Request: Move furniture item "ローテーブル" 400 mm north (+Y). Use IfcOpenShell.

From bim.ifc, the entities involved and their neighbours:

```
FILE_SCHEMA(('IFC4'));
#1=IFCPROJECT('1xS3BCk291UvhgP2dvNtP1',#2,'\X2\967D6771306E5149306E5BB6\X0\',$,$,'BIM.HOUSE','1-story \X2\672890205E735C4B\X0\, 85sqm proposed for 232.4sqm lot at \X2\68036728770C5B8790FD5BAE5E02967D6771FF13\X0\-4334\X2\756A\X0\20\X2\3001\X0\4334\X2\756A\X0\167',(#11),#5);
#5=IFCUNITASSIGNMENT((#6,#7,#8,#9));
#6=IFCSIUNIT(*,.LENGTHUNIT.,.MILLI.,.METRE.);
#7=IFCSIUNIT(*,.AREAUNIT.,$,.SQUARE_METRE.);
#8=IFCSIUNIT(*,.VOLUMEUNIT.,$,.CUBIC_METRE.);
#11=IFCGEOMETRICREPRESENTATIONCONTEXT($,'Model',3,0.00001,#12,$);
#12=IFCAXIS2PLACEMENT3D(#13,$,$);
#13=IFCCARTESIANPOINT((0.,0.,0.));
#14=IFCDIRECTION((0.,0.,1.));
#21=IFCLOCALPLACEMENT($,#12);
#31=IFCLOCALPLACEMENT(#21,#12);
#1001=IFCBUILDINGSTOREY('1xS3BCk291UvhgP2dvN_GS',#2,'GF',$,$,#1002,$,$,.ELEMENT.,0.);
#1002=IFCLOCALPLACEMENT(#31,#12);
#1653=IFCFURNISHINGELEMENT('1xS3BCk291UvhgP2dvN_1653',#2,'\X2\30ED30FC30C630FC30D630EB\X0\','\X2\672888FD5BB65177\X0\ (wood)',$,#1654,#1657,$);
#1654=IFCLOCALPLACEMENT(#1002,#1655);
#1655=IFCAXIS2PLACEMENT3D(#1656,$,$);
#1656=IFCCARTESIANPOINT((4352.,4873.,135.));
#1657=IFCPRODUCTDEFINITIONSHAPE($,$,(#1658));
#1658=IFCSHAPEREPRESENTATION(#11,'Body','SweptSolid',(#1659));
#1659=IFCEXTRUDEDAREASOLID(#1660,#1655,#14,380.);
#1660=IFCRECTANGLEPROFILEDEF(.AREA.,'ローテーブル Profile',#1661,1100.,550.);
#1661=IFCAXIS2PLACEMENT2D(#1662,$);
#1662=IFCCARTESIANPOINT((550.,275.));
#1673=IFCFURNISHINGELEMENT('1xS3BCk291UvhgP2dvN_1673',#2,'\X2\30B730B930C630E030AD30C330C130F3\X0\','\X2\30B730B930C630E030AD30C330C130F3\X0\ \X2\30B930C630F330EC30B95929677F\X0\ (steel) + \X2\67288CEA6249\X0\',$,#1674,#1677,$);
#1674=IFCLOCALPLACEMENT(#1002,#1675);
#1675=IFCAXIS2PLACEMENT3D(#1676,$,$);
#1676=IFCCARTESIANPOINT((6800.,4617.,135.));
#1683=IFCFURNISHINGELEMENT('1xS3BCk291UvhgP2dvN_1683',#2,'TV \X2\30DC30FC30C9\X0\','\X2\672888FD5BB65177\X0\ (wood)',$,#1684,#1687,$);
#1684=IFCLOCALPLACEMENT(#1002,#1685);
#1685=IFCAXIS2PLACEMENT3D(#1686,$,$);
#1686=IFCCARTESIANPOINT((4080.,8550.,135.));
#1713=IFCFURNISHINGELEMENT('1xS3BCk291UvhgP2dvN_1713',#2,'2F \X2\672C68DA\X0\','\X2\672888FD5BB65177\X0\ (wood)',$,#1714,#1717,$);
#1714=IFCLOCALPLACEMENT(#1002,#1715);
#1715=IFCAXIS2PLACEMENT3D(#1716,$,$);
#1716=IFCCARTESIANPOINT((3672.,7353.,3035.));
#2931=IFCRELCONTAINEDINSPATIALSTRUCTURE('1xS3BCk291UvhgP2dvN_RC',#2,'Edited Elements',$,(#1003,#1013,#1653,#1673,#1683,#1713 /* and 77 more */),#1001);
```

```python
import ifcopenshell
import ifcopenshell.api.geometry
import ifcopenshell.util.placement
import ifcopenshell.util.unit

model = ifcopenshell.open("bim.ifc")
unit_scale = ifcopenshell.util.unit.calculate_unit_scale(model)

item = model.by_id(1653)
matrix = ifcopenshell.util.placement.get_local_placement(item.ObjectPlacement)
matrix[1, 3] += 0.4 / unit_scale
ifcopenshell.api.geometry.edit_object_placement(model, product=item, matrix=matrix, is_si=False)

print(ifcopenshell.util.placement.get_local_placement(item.ObjectPlacement).round(3) + 0.0)

model.write("bim_v2.ifc")
```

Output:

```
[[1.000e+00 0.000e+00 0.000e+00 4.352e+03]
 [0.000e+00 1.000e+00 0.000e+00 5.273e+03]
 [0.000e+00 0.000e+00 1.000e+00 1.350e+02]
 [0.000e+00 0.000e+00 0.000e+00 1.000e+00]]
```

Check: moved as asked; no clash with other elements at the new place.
